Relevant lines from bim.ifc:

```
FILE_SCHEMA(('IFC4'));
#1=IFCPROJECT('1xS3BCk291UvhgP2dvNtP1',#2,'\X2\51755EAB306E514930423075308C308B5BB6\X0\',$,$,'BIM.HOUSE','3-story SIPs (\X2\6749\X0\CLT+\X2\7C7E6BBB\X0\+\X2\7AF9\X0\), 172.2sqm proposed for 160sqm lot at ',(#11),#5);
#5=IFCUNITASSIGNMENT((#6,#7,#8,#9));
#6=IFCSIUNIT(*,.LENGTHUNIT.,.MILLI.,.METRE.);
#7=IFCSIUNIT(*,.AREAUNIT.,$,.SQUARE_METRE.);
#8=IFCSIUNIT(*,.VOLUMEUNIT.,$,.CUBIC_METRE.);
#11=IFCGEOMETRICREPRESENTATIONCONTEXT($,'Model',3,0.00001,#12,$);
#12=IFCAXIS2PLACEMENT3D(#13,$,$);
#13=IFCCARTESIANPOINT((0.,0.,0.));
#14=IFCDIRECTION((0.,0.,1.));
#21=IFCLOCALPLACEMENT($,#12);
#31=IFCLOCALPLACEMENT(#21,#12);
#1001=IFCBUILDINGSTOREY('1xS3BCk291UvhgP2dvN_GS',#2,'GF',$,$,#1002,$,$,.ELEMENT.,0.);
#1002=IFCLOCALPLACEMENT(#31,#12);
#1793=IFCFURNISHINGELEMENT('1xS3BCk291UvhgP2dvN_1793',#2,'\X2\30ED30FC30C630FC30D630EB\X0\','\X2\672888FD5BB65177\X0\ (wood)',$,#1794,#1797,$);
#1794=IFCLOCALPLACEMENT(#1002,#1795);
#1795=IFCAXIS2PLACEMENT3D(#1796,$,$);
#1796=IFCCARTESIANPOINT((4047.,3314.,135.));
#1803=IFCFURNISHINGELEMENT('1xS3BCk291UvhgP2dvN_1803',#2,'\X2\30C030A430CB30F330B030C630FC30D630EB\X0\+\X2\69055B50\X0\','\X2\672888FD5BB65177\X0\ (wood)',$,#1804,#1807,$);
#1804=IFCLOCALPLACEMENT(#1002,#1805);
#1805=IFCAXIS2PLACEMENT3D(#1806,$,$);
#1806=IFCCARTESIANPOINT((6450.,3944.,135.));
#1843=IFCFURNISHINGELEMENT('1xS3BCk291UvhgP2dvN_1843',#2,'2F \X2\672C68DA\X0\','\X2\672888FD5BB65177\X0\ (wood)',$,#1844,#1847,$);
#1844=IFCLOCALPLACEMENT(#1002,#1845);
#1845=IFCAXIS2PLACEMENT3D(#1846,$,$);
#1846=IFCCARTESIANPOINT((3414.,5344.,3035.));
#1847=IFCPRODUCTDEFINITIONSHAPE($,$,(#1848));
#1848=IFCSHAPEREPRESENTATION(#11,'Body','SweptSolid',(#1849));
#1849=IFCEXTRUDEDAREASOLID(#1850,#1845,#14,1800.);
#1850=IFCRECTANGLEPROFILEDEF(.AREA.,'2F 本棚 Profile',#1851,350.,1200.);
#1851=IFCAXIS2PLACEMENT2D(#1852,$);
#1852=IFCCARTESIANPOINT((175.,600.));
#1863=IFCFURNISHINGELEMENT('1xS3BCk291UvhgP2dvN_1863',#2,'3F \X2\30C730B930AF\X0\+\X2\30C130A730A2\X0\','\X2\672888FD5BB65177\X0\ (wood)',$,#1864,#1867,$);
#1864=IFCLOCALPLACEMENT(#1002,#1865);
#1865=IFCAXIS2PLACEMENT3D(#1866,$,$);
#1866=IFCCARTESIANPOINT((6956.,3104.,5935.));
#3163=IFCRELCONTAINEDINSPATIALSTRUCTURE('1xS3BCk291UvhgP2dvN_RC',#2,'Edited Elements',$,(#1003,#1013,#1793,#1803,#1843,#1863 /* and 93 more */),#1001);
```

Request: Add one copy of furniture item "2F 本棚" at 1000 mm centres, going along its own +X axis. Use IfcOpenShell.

```python
import ifcopenshell
import ifcopenshell.api.geometry
import ifcopenshell.api.root
import ifcopenshell.util.element
import ifcopenshell.util.placement
import ifcopenshell.util.unit

model = ifcopenshell.open("bim.ifc")
unit_scale = ifcopenshell.util.unit.calculate_unit_scale(model)


def reuse_history(source, copy):
    """copy_class also copies each property set's owner history, people and application; keep the originals."""
    for rel in copy.IsDefinedBy:
        if rel.is_a("IfcRelDefinesByProperties") and (history := rel.RelatingPropertyDefinition.OwnerHistory):
            rel.RelatingPropertyDefinition.OwnerHistory = source.OwnerHistory
            ifcopenshell.util.element.remove_deep2(model, history)


source = model.by_id(1843)
base = ifcopenshell.util.placement.get_local_placement(source.ObjectPlacement)
step = base[:3, 0] * 1 / unit_scale

for i in range(1, 2):
    copy = ifcopenshell.api.root.copy_class(model, product=source)
    copy.Representation = ifcopenshell.util.element.copy_deep(
        model, source.Representation, exclude=["IfcGeometricRepresentationContext", "IfcRepresentationMap"]
    )
    reuse_history(source, copy)
    matrix = base.copy()
    matrix[:3, 3] += i * step
    print("added at", matrix[:3, 3].round(3) + 0.0)
    ifcopenshell.api.geometry.edit_object_placement(model, product=copy, matrix=matrix, is_si=False)

model.write("bim-out.ifc")
```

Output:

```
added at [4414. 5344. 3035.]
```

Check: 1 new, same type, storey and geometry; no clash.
